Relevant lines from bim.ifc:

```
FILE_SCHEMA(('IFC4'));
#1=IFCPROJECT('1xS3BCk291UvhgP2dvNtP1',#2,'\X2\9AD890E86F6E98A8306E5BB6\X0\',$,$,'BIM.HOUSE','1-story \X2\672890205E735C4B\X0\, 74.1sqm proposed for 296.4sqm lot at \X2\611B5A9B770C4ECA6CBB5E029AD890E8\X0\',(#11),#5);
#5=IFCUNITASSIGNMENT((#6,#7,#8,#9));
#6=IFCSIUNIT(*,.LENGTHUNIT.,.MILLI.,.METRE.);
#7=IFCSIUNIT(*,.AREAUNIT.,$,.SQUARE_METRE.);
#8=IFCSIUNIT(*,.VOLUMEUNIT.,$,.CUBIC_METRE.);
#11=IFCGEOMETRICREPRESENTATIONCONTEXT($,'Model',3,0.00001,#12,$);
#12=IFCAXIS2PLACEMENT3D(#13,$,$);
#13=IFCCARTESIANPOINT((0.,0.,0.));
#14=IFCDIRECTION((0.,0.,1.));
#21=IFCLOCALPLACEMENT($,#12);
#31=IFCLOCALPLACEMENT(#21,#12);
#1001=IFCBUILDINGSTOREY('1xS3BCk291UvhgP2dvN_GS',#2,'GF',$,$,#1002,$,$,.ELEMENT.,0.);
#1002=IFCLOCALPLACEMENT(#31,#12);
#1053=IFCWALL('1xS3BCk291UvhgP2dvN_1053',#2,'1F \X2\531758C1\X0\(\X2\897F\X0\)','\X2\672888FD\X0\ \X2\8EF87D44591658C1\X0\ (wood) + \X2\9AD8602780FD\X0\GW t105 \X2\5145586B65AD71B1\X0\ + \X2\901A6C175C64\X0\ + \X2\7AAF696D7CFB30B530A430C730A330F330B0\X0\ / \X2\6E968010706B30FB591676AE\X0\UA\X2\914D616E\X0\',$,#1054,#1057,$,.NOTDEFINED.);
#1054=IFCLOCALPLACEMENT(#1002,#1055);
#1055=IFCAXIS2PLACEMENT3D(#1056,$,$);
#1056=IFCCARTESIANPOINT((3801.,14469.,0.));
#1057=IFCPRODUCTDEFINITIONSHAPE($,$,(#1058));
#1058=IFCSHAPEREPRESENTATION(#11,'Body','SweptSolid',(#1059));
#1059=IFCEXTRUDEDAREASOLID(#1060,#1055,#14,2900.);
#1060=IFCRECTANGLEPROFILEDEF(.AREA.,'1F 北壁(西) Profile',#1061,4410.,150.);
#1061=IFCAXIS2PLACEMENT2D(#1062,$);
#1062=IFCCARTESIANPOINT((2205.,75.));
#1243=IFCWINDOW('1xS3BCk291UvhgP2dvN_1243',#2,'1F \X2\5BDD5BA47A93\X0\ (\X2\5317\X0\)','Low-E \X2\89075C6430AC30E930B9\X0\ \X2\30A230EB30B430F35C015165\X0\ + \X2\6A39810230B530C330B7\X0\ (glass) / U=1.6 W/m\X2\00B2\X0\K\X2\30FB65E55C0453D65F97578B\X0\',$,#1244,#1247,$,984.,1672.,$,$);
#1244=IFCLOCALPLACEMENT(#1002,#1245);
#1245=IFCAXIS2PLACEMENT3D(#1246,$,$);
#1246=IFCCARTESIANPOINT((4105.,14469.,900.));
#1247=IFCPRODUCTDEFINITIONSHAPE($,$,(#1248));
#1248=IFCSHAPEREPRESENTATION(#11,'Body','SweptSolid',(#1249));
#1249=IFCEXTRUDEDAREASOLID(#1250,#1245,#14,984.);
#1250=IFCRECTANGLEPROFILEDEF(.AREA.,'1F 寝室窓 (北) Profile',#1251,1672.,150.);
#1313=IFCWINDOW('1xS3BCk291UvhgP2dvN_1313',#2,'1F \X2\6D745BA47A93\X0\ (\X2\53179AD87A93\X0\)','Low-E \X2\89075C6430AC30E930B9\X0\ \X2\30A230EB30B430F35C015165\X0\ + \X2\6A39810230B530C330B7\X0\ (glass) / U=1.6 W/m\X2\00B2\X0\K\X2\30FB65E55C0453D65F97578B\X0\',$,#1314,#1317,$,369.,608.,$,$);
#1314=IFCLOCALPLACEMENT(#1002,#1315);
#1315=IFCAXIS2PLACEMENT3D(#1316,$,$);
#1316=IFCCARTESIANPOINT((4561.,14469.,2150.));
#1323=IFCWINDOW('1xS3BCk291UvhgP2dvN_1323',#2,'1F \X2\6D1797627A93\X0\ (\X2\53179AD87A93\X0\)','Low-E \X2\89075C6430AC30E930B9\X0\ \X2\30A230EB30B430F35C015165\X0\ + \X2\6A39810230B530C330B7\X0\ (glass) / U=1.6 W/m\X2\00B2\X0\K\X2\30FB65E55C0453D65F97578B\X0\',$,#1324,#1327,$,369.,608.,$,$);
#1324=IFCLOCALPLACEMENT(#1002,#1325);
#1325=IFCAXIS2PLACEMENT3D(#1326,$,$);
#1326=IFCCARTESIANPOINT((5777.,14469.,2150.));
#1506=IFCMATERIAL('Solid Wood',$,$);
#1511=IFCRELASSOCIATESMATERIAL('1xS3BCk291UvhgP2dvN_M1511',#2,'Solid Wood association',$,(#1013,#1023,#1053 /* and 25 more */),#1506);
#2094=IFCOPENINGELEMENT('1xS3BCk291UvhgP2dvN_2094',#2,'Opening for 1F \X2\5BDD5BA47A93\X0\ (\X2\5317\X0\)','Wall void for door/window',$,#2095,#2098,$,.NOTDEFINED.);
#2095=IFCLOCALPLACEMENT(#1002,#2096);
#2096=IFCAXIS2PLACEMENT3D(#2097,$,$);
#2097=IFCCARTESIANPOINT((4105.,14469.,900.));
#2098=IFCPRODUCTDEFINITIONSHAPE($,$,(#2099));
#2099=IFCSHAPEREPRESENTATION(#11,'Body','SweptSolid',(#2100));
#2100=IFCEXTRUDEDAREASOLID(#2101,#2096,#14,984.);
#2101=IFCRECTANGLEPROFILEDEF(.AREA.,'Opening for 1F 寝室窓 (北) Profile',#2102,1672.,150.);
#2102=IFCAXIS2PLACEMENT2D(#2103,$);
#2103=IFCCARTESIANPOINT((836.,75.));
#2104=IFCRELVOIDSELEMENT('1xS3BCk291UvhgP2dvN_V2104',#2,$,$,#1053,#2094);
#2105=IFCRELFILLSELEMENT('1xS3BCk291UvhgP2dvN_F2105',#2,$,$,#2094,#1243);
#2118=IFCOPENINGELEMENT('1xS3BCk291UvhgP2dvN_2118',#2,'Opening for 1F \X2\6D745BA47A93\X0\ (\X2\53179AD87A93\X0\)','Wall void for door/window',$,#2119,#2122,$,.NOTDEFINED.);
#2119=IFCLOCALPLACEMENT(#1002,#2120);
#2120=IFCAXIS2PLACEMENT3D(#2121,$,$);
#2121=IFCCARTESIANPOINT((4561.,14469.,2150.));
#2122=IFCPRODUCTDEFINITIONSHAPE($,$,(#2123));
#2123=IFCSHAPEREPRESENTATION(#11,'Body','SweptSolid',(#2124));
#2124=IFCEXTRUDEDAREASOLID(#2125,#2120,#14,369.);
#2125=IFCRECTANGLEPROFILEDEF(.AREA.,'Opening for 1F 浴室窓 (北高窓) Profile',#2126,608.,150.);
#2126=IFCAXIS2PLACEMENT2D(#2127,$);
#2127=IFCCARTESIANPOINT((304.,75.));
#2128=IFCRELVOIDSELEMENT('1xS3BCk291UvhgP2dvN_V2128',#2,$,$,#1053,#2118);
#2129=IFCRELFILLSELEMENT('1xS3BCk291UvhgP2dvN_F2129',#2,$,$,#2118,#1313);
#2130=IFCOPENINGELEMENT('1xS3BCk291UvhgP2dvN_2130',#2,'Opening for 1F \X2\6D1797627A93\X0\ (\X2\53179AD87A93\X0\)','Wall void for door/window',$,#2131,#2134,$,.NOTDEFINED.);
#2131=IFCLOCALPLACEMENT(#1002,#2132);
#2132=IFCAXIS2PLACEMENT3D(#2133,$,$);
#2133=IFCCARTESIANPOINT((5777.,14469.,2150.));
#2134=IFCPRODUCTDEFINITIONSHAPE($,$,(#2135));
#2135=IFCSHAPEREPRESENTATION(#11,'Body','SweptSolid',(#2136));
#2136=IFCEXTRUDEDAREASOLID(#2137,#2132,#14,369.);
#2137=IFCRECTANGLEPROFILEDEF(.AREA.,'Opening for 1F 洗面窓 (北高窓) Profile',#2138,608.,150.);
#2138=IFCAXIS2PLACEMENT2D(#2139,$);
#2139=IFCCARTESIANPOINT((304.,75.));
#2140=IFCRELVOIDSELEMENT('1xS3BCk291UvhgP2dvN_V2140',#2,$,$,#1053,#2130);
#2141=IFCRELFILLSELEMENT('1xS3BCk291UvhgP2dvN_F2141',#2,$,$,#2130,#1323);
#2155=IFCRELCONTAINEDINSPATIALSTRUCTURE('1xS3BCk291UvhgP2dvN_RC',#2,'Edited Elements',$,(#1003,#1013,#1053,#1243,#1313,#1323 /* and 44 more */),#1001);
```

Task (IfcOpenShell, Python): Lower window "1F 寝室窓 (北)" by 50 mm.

```python
import numpy as np
import ifcopenshell
import ifcopenshell.api.geometry
import ifcopenshell.util.placement
import ifcopenshell.util.unit

model = ifcopenshell.open("bim.ifc")
unit_scale = ifcopenshell.util.unit.calculate_unit_scale(model)

window = model.by_guid("1xS3BCk291UvhgP2dvN_1243")
opening = window.FillsVoids[0].RelatingOpeningElement
dz = -0.05 / unit_scale

shift = np.array([0.0, 0.0, dz])
# The window is not placed relative to its opening, so move both.
for product in (opening, window):
    matrix = ifcopenshell.util.placement.get_local_placement(product.ObjectPlacement)
    matrix[:3, 3] += shift
    ifcopenshell.api.geometry.edit_object_placement(model, product=product, matrix=matrix, is_si=False)

print(f"moved by {dz * unit_scale:+.3f} m")

model.write("bim_rev.ifc")
```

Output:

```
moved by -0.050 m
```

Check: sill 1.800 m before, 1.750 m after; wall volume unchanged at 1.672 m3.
